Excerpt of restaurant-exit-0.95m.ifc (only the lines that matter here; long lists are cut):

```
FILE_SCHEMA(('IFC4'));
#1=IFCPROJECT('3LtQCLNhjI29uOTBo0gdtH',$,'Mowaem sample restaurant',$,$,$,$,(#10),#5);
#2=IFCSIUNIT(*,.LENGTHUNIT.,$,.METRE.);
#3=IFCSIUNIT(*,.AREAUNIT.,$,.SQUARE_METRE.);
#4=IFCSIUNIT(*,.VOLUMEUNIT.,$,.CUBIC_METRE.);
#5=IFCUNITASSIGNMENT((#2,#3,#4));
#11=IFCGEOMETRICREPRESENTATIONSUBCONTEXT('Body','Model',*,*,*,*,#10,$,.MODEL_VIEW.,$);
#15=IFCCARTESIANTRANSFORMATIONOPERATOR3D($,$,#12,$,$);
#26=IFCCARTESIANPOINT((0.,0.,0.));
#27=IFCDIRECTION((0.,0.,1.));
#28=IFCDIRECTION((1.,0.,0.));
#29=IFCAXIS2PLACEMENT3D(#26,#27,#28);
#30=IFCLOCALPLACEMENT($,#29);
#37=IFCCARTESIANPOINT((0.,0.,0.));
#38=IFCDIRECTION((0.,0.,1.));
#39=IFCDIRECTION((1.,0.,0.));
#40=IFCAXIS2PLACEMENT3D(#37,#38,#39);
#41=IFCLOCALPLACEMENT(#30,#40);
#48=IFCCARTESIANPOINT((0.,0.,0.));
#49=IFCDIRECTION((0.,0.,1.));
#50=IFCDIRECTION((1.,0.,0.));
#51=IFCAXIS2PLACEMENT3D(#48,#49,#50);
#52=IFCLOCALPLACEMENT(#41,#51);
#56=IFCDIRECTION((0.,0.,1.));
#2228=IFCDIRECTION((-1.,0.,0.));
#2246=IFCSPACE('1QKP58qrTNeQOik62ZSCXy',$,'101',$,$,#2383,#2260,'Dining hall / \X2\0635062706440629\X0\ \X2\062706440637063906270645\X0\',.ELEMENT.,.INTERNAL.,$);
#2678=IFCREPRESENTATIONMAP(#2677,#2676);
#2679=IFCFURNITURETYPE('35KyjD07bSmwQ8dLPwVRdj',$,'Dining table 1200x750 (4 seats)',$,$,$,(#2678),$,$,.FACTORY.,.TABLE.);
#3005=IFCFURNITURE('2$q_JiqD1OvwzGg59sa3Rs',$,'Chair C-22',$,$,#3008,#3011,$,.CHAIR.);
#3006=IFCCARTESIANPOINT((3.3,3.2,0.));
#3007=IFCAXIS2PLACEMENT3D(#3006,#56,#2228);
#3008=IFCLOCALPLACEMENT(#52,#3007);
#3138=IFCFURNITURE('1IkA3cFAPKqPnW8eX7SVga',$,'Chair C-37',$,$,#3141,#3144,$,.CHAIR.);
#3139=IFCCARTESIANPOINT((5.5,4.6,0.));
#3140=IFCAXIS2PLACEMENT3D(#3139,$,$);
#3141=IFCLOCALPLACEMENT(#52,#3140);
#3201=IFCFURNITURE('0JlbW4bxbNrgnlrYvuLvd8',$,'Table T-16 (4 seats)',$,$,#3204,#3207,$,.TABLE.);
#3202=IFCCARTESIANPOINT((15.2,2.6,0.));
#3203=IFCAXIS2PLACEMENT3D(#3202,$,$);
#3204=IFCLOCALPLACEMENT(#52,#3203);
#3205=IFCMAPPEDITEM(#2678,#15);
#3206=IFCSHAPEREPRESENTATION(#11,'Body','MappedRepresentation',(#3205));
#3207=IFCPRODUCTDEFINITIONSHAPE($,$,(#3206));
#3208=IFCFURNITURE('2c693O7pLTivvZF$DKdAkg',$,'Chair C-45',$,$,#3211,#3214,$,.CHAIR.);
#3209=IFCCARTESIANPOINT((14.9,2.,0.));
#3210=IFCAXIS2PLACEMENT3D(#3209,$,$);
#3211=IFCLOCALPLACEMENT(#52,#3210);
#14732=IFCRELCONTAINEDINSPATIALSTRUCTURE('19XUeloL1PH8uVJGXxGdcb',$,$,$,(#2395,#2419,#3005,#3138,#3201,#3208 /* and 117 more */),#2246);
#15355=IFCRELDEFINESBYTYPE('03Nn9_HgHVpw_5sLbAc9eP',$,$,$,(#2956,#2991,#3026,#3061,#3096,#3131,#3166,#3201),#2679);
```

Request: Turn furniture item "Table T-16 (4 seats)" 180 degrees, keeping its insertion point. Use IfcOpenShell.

```python
import ifcopenshell
import ifcopenshell.api.geometry
import ifcopenshell.util.placement

model = ifcopenshell.open("restaurant-exit-0.95m.ifc")

item = model.by_guid("0JlbW4bxbNrgnlrYvuLvd8")
matrix = ifcopenshell.util.placement.get_local_placement(item.ObjectPlacement)
matrix = matrix @ ifcopenshell.util.placement.rotation(180, "Z")
ifcopenshell.api.geometry.edit_object_placement(model, product=item, matrix=matrix, is_si=False)

print(ifcopenshell.util.placement.get_local_placement(item.ObjectPlacement).round(3) + 0.0)

model.write("restaurant-exit-0.95m_updated.ifc")
```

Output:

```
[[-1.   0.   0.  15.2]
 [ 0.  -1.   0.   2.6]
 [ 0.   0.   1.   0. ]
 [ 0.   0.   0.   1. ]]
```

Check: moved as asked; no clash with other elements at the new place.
